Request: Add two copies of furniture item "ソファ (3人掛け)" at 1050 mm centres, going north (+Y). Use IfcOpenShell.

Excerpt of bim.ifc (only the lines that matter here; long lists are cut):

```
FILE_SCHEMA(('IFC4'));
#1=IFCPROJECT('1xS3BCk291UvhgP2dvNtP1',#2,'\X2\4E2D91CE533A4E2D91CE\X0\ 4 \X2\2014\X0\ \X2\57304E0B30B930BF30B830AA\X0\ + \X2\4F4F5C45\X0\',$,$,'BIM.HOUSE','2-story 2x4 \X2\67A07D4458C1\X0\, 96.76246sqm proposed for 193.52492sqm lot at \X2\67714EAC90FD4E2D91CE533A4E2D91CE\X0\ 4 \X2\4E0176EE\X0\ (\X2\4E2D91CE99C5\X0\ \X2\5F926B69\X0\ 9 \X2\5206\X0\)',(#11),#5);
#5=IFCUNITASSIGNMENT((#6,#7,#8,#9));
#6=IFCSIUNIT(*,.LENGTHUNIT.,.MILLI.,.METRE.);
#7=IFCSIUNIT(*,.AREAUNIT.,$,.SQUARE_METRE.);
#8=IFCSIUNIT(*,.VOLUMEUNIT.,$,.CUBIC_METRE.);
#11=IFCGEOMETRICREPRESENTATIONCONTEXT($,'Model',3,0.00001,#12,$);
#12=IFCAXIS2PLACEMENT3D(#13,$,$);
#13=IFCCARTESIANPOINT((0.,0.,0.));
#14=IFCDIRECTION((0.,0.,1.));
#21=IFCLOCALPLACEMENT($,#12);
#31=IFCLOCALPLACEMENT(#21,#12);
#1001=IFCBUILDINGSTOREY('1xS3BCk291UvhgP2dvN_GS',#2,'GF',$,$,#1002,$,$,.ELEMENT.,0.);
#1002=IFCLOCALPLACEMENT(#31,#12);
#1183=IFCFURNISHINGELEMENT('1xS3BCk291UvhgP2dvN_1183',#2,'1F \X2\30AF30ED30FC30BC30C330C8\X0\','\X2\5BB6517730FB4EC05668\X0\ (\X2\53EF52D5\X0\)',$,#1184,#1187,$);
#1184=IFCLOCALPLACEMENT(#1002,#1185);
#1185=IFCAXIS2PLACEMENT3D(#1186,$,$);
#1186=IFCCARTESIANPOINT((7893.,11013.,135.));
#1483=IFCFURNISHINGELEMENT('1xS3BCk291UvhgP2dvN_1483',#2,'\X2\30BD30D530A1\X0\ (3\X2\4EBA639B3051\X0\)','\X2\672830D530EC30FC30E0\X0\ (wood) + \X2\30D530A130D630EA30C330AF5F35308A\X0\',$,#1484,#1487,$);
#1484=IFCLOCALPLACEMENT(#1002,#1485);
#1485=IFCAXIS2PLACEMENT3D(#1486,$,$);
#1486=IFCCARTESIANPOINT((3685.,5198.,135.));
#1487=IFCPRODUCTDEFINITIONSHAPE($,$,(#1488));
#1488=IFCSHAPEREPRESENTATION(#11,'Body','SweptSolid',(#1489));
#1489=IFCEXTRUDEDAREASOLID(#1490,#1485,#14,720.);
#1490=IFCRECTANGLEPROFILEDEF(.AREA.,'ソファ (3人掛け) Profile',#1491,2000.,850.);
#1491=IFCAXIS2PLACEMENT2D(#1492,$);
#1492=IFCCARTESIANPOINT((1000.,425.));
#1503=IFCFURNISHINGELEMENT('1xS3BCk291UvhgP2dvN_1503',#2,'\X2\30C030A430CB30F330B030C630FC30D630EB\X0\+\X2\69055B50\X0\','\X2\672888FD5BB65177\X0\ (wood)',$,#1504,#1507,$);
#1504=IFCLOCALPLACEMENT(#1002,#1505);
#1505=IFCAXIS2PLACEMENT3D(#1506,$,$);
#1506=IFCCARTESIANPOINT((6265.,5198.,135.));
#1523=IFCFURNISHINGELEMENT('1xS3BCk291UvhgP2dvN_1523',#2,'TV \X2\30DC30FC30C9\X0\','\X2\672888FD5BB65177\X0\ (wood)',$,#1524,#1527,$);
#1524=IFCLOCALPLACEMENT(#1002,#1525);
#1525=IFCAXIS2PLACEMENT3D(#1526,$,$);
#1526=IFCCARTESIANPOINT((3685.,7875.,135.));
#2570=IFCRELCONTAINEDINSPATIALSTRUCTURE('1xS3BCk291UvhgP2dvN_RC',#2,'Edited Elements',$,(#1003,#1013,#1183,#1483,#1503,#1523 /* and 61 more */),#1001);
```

```python
import numpy as np
import ifcopenshell
import ifcopenshell.api.geometry
import ifcopenshell.api.root
import ifcopenshell.util.element
import ifcopenshell.util.placement
import ifcopenshell.util.unit

model = ifcopenshell.open("bim.ifc")
unit_scale = ifcopenshell.util.unit.calculate_unit_scale(model)


def reuse_history(source, copy):
    """copy_class also copies each property set's owner history, people and application; keep the originals."""
    for rel in copy.IsDefinedBy:
        if rel.is_a("IfcRelDefinesByProperties") and (history := rel.RelatingPropertyDefinition.OwnerHistory):
            rel.RelatingPropertyDefinition.OwnerHistory = source.OwnerHistory
            ifcopenshell.util.element.remove_deep2(model, history)


source = model.by_guid("1xS3BCk291UvhgP2dvN_1483")
base = ifcopenshell.util.placement.get_local_placement(source.ObjectPlacement)
step = np.array([0.0, 1.0, 0.0]) * 1.05 / unit_scale

for i in range(1, 3):
    copy = ifcopenshell.api.root.copy_class(model, product=source)
    copy.Representation = ifcopenshell.util.element.copy_deep(
        model, source.Representation, exclude=["IfcGeometricRepresentationContext", "IfcRepresentationMap"]
    )
    reuse_history(source, copy)
    matrix = base.copy()
    matrix[:3, 3] += i * step
    print("added at", matrix[:3, 3].round(3) + 0.0)
    ifcopenshell.api.geometry.edit_object_placement(model, product=copy, matrix=matrix, is_si=False)

model.write("bim_edited.ifc")
```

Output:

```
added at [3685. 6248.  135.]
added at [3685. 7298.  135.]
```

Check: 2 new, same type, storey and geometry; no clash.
